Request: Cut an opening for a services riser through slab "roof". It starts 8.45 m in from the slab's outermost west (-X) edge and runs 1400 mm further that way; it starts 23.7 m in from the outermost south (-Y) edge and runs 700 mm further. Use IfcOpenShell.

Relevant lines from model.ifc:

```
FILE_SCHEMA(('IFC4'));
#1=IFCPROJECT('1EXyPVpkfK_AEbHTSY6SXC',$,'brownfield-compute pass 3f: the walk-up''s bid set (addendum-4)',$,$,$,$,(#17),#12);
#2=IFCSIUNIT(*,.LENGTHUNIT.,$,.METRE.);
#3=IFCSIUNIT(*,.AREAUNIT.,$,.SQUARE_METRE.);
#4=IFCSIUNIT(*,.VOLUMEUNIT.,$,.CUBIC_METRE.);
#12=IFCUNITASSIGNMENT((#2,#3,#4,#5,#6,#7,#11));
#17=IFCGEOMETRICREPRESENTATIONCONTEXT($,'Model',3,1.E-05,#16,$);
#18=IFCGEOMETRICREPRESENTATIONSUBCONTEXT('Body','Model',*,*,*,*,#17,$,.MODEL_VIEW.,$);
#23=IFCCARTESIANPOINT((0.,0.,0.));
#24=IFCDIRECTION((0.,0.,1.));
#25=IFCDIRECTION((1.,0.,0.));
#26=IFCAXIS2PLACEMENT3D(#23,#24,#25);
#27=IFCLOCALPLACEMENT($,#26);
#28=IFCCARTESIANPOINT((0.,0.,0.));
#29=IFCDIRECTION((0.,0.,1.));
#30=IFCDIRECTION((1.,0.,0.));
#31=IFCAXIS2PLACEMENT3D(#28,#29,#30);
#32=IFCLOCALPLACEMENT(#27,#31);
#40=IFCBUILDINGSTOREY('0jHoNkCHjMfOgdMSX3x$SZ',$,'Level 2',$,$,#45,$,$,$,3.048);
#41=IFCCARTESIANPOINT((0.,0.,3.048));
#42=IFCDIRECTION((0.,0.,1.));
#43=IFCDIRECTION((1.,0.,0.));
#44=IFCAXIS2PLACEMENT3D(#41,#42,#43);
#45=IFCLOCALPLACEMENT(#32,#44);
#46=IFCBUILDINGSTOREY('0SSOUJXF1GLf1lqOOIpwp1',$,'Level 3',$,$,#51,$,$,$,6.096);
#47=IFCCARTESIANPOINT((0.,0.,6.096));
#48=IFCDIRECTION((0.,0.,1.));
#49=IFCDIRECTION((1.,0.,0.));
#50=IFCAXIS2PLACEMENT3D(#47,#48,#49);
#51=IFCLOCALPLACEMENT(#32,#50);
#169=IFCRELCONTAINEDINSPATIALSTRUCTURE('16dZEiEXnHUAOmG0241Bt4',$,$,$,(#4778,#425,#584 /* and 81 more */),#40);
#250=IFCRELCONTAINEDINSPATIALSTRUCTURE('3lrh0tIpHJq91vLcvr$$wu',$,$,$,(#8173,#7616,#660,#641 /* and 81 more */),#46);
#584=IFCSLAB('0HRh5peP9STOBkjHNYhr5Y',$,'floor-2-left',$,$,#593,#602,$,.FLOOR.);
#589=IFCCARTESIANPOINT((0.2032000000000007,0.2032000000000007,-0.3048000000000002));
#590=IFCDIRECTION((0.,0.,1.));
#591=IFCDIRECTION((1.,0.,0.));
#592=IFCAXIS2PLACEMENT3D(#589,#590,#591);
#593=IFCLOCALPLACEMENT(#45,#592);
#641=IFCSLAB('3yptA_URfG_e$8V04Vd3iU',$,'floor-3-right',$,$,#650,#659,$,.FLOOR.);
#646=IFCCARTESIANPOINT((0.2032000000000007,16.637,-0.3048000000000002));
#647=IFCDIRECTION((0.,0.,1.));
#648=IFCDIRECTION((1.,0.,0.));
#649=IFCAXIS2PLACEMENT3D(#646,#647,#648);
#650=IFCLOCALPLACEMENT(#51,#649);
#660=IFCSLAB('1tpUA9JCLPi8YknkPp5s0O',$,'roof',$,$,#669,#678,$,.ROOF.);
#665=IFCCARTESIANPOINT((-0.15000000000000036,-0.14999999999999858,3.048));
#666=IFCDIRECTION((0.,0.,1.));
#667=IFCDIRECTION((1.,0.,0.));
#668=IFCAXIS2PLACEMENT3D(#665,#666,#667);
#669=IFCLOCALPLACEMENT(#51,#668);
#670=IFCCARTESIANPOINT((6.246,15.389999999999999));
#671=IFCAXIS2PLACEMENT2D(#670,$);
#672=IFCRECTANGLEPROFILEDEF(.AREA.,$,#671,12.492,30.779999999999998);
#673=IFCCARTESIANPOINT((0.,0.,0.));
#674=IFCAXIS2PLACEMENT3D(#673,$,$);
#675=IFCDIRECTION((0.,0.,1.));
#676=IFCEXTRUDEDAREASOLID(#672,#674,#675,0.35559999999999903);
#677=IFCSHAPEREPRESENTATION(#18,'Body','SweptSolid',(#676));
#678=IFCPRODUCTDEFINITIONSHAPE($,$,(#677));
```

```python
import numpy as np
import ifcopenshell
import ifcopenshell.api.feature
import ifcopenshell.api.geometry
import ifcopenshell.api.root
import ifcopenshell.geom
import ifcopenshell.util.placement
import ifcopenshell.util.representation
import ifcopenshell.util.shape
import ifcopenshell.util.unit

model = ifcopenshell.open("model.ifc")
unit_scale = ifcopenshell.util.unit.calculate_unit_scale(model)
settings = ifcopenshell.geom.settings()


def volume(element):
    """Net volume in cubic metres, openings subtracted."""
    shape = ifcopenshell.geom.create_shape(settings, element)
    return ifcopenshell.util.shape.get_volume(shape.geometry)


slab = model.by_guid("1tpUA9JCLPi8YknkPp5s0O")
before = volume(slab)

# Extent in the slab's own axes, in metres. The edges named are its -X and -Y sides.
slab_shape = ifcopenshell.geom.create_shape(settings, slab)
vertices = ifcopenshell.util.shape.get_vertices(slab_shape.geometry)
x_min, y_min, bottom = vertices.min(axis=0)
top = vertices[:, 2].max()

opening = ifcopenshell.api.root.create_entity(model, ifc_class="IfcOpeningElement", name="Services riser opening", predefined_type="OPENING")
context = ifcopenshell.util.representation.get_context(model, "Model", "Body", "MODEL_VIEW")
width, depth = 1.4, 0.7
outline = [(0.0, 0.0), (width, 0.0), (width, depth), (0.0, depth), (0.0, 0.0)]
# Overshoot both faces by 50 mm so the cut is clean.
shape = ifcopenshell.api.geometry.add_slab_representation(
    model, context=context, depth=top - bottom + 0.1, polyline=outline
)
ifcopenshell.api.geometry.assign_representation(model, product=opening, representation=shape)

matrix = ifcopenshell.util.placement.get_local_placement(slab.ObjectPlacement)
matrix[:, 3] = matrix @ np.append(np.array([x_min + 8.45, y_min + 23.7, bottom - 0.05]) / unit_scale, 1.0)
ifcopenshell.api.geometry.edit_object_placement(model, product=opening, matrix=matrix, is_si=False)
ifcopenshell.api.feature.add_feature(model, feature=opening, element=slab)

after = volume(slab)

print(f"slab volume {before:.3f} -> {after:.3f} m3")

model.write("model-out.ifc")
```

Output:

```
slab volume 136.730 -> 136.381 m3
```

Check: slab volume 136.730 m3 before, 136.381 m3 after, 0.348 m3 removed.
